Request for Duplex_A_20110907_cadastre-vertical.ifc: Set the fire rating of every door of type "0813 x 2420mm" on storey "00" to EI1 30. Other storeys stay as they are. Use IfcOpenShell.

First a look at what the model holds.

```python
import ifcopenshell
import ifcopenshell.util.element

model = ifcopenshell.open("Duplex_A_20110907_cadastre-vertical.ifc")
print(model.schema)
storey = next(s for s in model.by_type("IfcBuildingStorey") if s.Name == "00")
doors = [e for e in ifcopenshell.util.element.get_decomposition(storey) if e.is_a("IfcDoor")]
seen = {}
for e in doors:
    element_type = ifcopenshell.util.element.get_type(e)
    key = (element_type.Name if element_type != e and element_type else None, ifcopenshell.util.element.get_pset(e, "Pset_DoorCommon", "FireRating"))
    seen[key] = seen.get(key, 0) + 1
for (name, value), count in sorted(seen.items(), key=str):
    print(count, "x", name, "|", value)
```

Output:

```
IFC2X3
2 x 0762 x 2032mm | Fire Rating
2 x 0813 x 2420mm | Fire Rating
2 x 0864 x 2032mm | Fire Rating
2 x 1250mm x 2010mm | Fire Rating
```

```python
import ifcopenshell
import ifcopenshell.api.pset
import ifcopenshell.util.element

model = ifcopenshell.open("Duplex_A_20110907_cadastre-vertical.ifc")

storey = next(s for s in model.by_type("IfcBuildingStorey") if s.Name == "00")
doors = [e for e in ifcopenshell.util.element.get_decomposition(storey) if e.is_a("IfcDoor")]

count = 0
for e in doors:
    element_type = ifcopenshell.util.element.get_type(e)
    if element_type in (None, e) or element_type.Name != "0813 x 2420mm":
        continue
    # add_pset returns the element's existing set when there is one.
    pset = ifcopenshell.api.pset.add_pset(model, product=e, name="Pset_DoorCommon")
    ifcopenshell.api.pset.edit_pset(model, pset=pset, properties={"FireRating": "EI1 30"})
    count += 1

print(count, "doors updated")

model.write("Duplex_A_20110907_cadastre-vertical_v2.ifc")
```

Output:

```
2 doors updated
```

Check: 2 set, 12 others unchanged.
